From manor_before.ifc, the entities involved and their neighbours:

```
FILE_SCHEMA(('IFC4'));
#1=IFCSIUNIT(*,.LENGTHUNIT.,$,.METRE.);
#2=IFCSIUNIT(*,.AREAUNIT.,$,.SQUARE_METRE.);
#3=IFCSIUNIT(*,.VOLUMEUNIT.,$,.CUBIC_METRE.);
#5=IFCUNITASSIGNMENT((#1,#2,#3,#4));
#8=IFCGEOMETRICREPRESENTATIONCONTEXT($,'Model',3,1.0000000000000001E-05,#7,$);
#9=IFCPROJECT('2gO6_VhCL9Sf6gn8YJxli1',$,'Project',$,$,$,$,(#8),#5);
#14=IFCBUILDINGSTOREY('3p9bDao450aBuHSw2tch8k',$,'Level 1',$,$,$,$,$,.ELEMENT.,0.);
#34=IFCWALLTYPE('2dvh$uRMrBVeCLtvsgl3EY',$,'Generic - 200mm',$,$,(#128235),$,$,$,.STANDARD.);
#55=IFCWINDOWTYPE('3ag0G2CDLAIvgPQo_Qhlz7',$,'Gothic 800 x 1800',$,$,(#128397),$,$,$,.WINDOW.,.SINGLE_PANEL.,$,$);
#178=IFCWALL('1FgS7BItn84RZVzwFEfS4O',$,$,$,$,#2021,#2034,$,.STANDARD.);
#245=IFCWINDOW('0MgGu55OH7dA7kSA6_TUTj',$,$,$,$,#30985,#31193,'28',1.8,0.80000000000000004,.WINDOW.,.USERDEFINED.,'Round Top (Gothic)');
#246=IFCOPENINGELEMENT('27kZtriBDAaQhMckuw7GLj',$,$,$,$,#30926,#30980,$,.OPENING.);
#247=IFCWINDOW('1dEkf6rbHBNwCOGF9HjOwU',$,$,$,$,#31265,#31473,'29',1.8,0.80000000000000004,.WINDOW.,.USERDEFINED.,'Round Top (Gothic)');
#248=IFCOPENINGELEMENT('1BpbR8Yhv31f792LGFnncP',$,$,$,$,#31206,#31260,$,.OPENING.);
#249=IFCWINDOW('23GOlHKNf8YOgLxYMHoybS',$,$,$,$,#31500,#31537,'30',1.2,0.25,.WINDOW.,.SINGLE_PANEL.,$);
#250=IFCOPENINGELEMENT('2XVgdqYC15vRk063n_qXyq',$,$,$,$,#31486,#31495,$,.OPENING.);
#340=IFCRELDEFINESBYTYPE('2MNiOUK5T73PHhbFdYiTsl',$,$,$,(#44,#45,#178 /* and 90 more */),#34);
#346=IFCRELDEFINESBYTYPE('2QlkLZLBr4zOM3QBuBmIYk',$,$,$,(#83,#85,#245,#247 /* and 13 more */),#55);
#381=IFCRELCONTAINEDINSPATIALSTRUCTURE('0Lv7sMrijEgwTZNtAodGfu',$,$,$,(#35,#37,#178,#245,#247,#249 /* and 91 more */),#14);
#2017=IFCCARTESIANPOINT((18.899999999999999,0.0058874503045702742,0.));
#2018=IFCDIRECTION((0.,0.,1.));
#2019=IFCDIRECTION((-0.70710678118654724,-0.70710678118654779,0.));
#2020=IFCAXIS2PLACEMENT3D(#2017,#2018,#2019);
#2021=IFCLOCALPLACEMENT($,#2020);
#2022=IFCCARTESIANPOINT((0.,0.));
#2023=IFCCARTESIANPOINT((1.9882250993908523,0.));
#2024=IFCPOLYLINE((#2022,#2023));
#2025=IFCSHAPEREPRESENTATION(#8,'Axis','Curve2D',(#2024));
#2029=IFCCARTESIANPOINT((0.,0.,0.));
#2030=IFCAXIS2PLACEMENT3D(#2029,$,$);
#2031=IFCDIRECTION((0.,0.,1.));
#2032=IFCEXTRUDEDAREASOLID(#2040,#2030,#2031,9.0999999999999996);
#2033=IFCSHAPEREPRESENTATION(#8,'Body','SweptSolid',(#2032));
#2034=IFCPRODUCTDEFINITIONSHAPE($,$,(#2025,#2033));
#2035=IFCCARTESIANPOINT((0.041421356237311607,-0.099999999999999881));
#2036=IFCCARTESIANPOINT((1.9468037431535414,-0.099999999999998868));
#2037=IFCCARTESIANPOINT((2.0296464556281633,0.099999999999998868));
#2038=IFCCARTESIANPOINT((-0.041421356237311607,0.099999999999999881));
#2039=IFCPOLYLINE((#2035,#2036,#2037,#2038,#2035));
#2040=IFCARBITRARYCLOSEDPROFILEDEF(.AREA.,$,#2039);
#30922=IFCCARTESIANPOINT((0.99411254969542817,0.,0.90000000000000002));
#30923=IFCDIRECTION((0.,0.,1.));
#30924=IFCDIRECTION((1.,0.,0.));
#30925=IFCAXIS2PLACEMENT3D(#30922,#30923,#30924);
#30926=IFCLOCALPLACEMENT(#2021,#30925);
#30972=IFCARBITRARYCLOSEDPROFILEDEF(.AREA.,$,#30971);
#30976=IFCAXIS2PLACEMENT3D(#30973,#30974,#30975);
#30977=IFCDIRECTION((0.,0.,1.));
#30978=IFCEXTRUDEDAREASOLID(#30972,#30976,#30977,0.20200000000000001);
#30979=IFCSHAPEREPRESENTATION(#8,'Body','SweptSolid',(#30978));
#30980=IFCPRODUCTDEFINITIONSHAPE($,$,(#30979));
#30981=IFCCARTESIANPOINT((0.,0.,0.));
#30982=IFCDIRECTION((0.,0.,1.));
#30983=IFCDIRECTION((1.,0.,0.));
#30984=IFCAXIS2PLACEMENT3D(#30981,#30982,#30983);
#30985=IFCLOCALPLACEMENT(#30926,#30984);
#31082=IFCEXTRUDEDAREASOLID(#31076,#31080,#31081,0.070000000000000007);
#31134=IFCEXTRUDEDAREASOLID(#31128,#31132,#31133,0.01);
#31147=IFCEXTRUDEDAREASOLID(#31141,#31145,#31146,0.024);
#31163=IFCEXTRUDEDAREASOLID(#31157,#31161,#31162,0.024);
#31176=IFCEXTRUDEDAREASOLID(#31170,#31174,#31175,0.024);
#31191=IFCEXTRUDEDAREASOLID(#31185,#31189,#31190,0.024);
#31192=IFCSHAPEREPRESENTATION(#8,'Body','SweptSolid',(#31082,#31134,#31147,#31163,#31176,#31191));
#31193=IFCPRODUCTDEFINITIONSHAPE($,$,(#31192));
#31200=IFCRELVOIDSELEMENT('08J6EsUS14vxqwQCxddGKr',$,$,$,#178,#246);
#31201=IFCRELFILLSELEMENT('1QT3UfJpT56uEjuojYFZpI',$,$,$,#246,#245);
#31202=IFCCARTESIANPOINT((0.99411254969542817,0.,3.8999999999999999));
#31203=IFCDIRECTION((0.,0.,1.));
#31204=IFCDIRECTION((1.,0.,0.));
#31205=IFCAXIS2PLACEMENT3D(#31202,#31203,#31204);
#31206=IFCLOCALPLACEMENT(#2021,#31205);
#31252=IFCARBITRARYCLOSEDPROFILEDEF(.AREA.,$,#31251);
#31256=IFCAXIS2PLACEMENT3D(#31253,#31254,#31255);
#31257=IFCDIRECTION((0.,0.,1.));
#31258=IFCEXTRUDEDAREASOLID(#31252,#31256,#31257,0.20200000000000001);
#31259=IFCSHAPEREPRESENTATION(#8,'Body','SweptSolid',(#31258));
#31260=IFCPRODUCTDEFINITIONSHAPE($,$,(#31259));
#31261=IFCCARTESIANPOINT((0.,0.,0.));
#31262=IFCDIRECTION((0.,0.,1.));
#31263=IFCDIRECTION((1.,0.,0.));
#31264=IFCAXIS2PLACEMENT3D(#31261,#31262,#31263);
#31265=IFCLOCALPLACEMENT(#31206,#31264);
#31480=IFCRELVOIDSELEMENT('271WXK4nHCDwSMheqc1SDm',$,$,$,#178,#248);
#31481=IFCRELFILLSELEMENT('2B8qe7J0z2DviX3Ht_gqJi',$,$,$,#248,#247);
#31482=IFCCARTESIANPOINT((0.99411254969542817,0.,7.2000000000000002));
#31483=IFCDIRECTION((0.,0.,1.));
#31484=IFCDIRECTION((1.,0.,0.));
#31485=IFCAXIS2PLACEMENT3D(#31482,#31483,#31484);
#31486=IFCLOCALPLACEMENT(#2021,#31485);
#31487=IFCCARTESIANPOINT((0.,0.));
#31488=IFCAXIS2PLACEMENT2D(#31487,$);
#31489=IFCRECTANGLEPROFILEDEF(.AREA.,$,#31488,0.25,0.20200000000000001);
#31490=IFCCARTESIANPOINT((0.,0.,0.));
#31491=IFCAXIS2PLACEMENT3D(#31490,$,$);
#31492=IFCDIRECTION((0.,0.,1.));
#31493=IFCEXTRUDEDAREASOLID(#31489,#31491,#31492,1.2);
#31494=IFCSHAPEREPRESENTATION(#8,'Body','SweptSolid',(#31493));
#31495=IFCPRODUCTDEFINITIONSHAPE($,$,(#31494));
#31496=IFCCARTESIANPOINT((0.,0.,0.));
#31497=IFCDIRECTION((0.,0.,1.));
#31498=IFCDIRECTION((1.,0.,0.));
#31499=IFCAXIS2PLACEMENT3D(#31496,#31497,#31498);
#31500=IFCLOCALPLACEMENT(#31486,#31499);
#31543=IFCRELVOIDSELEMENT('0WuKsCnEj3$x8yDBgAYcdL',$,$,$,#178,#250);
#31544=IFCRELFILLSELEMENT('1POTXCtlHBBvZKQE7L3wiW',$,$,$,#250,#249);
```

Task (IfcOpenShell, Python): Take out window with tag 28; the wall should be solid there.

```python
import ifcopenshell
import ifcopenshell.api.feature
import ifcopenshell.api.root
import ifcopenshell.geom
import ifcopenshell.util.shape

model = ifcopenshell.open("manor_before.ifc")
settings = ifcopenshell.geom.settings()


def volume(element):
    """Net volume in cubic metres, openings subtracted."""
    shape = ifcopenshell.geom.create_shape(settings, element)
    return ifcopenshell.util.shape.get_volume(shape.geometry)


window = model.by_guid("0MgGu55OH7dA7kSA6_TUTj")
opening = window.FillsVoids[0].RelatingOpeningElement
wall = opening.VoidsElements[0].RelatingBuildingElement
before = volume(wall)

ifcopenshell.api.root.remove_product(model, product=window)
ifcopenshell.api.feature.remove_feature(model, feature=opening)

after = volume(wall)

print(f"wall volume {before:.3f} -> {after:.3f} m3")

model.write("manor_before_edited.ifc")
```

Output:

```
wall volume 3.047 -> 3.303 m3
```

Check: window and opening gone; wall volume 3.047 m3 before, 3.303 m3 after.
